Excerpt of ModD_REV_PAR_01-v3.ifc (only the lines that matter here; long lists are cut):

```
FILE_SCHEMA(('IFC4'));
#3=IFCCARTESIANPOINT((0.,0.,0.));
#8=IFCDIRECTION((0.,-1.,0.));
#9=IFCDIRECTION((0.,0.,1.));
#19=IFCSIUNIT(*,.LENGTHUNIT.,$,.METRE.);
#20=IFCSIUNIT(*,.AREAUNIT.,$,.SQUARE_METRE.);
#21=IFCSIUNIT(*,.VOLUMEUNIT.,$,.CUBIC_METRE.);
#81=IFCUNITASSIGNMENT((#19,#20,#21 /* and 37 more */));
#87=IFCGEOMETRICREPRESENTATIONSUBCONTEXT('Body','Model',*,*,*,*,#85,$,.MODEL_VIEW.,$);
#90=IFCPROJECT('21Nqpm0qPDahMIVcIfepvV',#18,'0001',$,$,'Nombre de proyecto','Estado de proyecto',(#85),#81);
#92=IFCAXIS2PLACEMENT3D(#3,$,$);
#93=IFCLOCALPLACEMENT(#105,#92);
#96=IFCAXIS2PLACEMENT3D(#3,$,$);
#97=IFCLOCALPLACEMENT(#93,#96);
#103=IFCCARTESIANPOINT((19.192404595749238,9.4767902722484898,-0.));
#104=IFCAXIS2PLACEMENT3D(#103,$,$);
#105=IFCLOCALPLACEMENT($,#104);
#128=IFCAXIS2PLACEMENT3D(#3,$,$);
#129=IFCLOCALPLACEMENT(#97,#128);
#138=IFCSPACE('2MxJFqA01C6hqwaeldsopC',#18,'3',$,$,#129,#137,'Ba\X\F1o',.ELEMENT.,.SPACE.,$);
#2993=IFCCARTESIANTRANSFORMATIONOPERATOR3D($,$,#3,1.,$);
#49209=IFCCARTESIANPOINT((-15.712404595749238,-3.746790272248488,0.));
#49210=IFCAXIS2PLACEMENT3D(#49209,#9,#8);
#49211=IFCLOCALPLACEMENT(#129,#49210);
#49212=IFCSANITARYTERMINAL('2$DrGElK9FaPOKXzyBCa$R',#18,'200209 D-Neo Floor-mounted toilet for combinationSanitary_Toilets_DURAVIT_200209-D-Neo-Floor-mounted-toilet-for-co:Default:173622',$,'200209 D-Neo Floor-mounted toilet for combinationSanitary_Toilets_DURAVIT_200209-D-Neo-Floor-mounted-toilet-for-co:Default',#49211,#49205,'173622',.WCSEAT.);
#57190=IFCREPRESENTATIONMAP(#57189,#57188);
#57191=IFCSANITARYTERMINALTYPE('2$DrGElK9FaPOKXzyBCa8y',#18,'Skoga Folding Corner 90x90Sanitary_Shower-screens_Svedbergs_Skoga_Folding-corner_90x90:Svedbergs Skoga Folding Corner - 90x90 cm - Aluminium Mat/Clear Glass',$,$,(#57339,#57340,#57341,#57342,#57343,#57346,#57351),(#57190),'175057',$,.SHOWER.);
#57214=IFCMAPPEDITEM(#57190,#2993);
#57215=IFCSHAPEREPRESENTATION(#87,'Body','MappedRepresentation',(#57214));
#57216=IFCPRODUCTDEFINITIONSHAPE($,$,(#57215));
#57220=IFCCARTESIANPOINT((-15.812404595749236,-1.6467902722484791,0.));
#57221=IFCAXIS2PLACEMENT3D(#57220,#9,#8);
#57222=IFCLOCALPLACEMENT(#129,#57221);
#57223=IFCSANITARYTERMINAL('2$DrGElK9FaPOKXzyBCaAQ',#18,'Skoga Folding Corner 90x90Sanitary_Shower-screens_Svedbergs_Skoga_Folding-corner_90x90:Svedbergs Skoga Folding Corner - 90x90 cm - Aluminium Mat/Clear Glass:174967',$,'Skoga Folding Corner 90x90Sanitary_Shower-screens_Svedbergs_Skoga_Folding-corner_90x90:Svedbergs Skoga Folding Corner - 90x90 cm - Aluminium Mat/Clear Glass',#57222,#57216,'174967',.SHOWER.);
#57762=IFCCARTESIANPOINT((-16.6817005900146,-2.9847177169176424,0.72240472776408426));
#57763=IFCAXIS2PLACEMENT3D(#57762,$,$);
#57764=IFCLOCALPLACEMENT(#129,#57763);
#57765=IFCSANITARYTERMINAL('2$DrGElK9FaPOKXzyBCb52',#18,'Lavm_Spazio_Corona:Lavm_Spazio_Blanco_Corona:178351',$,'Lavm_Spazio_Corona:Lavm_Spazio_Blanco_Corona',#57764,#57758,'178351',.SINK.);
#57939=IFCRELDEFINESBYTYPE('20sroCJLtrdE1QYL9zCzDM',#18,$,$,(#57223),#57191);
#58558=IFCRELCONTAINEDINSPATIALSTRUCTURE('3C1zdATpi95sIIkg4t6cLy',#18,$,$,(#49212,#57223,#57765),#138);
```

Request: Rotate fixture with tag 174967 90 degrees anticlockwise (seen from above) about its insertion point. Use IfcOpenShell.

```python
import ifcopenshell
import ifcopenshell.api.geometry
import ifcopenshell.util.placement

model = ifcopenshell.open("ModD_REV_PAR_01-v3.ifc")

item = model.by_guid("2$DrGElK9FaPOKXzyBCaAQ")
matrix = ifcopenshell.util.placement.get_local_placement(item.ObjectPlacement)
matrix = matrix @ ifcopenshell.util.placement.rotation(90, "Z")
ifcopenshell.api.geometry.edit_object_placement(model, product=item, matrix=matrix, is_si=False)

print(ifcopenshell.util.placement.get_local_placement(item.ObjectPlacement).round(3) + 0.0)

model.write("ModD_REV_PAR_01-v3_v2.ifc")
```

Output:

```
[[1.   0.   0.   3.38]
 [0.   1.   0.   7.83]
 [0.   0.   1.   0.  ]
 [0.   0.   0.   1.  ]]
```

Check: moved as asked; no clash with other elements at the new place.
